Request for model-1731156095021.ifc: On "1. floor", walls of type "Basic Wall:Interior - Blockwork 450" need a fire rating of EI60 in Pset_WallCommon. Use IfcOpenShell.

First a look at what the model holds.

```python
import ifcopenshell
import ifcopenshell.util.element

model = ifcopenshell.open("model-1731156095021.ifc")
print(model.schema)
storey = next(s for s in model.by_type("IfcBuildingStorey") if s.Name == "1. floor")
walls = [e for e in ifcopenshell.util.element.get_decomposition(storey) if e.is_a("IfcWall")]
seen = {}
for e in walls:
    element_type = ifcopenshell.util.element.get_type(e)
    key = (element_type.Name if element_type != e and element_type else None, ifcopenshell.util.element.get_pset(e, "Pset_WallCommon", "FireRating"))
    seen[key] = seen.get(key, 0) + 1
for (name, value), count in sorted(seen.items(), key=str):
    print(count, "x", name, "|", value)
```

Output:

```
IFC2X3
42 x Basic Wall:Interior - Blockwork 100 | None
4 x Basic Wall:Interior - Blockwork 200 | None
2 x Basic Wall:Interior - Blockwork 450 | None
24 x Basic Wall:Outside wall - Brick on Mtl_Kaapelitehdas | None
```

```python
import ifcopenshell
import ifcopenshell.api.pset
import ifcopenshell.util.element

model = ifcopenshell.open("model-1731156095021.ifc")

storey = next(s for s in model.by_type("IfcBuildingStorey") if s.Name == "1. floor")
walls = [e for e in ifcopenshell.util.element.get_decomposition(storey) if e.is_a("IfcWall")]

count = 0
for e in walls:
    element_type = ifcopenshell.util.element.get_type(e)
    if element_type in (None, e) or element_type.Name != "Basic Wall:Interior - Blockwork 450":
        continue
    # add_pset returns the element's existing set when there is one.
    pset = ifcopenshell.api.pset.add_pset(model, product=e, name="Pset_WallCommon")
    ifcopenshell.api.pset.edit_pset(model, pset=pset, properties={"FireRating": "EI60"})
    count += 1

print(count, "walls updated")

model.write("model-1731156095021_edited.ifc")
```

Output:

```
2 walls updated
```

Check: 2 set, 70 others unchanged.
